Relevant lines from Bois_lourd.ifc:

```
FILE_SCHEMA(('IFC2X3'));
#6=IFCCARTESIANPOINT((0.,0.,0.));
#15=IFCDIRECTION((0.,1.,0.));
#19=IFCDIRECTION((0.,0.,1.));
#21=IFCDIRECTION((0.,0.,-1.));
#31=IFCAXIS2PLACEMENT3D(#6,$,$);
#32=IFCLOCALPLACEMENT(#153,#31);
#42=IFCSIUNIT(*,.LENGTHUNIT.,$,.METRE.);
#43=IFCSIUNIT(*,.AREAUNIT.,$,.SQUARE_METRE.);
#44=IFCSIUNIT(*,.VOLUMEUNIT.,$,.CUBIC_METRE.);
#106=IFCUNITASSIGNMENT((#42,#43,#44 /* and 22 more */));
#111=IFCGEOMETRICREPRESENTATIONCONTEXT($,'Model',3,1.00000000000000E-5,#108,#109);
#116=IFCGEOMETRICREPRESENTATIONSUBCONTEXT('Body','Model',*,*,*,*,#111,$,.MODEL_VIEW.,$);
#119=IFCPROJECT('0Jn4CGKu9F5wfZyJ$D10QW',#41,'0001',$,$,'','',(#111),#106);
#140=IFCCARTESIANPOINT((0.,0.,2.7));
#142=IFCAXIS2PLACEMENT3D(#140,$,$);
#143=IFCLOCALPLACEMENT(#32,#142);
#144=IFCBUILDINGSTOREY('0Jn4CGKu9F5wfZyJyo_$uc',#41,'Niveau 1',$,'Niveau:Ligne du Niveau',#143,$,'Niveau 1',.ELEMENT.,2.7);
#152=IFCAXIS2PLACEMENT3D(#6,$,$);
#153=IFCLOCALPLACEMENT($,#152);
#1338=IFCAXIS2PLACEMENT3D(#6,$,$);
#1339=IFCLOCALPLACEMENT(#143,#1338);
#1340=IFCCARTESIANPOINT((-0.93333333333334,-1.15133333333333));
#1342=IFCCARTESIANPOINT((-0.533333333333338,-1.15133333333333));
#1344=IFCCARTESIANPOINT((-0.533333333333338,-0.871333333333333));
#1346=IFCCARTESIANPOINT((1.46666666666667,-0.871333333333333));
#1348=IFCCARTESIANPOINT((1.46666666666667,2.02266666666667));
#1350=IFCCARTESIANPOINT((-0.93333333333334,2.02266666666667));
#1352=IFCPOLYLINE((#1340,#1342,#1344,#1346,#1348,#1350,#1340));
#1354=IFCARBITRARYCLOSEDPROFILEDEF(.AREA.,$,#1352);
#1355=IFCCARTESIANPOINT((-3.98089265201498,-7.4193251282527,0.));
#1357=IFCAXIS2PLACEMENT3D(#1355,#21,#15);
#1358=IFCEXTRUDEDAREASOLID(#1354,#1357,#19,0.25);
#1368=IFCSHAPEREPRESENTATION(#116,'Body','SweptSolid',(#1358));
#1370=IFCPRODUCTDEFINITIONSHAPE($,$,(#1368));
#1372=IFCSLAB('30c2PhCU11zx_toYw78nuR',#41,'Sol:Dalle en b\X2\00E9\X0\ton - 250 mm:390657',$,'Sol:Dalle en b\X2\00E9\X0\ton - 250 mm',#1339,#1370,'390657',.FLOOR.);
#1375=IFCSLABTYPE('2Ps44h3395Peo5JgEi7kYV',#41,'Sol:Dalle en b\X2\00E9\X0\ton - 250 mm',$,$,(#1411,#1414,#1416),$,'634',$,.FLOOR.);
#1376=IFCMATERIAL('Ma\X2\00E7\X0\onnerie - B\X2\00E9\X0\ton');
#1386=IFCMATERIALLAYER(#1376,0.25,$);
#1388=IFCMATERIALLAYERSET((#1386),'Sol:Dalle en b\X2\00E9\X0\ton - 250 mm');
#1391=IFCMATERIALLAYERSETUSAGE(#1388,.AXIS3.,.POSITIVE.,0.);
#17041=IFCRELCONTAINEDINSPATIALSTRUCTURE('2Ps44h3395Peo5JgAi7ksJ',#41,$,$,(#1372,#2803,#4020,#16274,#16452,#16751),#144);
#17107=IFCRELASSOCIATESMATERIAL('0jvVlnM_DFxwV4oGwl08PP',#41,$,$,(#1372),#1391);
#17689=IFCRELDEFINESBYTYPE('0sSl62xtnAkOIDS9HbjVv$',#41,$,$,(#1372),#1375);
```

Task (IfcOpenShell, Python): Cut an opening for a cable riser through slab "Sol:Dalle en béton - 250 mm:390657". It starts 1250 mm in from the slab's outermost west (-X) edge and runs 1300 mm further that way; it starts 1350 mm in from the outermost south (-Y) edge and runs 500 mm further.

```python
import numpy as np
import ifcopenshell
import ifcopenshell.api.feature
import ifcopenshell.api.geometry
import ifcopenshell.api.root
import ifcopenshell.geom
import ifcopenshell.util.placement
import ifcopenshell.util.representation
import ifcopenshell.util.shape
import ifcopenshell.util.unit

model = ifcopenshell.open("Bois_lourd.ifc")
unit_scale = ifcopenshell.util.unit.calculate_unit_scale(model)
settings = ifcopenshell.geom.settings()


def volume(element):
    """Net volume in cubic metres, openings subtracted."""
    shape = ifcopenshell.geom.create_shape(settings, element)
    return ifcopenshell.util.shape.get_volume(shape.geometry)


slab = model.by_guid("30c2PhCU11zx_toYw78nuR")
before = volume(slab)

# Extent in the slab's own axes, in metres. The edges named are its -X and -Y sides.
slab_shape = ifcopenshell.geom.create_shape(settings, slab)
vertices = ifcopenshell.util.shape.get_vertices(slab_shape.geometry)
x_min, y_min, bottom = vertices.min(axis=0)
top = vertices[:, 2].max()

opening = ifcopenshell.api.root.create_entity(model, ifc_class="IfcOpeningElement", name="Cable riser opening")
context = ifcopenshell.util.representation.get_context(model, "Model", "Body", "MODEL_VIEW")
width, depth = 1.3, 0.5
outline = [(0.0, 0.0), (width, 0.0), (width, depth), (0.0, depth), (0.0, 0.0)]
# Overshoot both faces by 50 mm so the cut is clean.
shape = ifcopenshell.api.geometry.add_slab_representation(
    model, context=context, depth=top - bottom + 0.1, polyline=outline
)
ifcopenshell.api.geometry.assign_representation(model, product=opening, representation=shape)

matrix = ifcopenshell.util.placement.get_local_placement(slab.ObjectPlacement)
matrix[:, 3] = matrix @ np.append(np.array([x_min + 1.25, y_min + 1.35, bottom - 0.05]) / unit_scale, 1.0)
ifcopenshell.api.geometry.edit_object_placement(model, product=opening, matrix=matrix, is_si=False)
ifcopenshell.api.feature.add_feature(model, feature=opening, element=slab)

after = volume(slab)

print(f"slab volume {before:.3f} -> {after:.3f} m3")

model.write("Bois_lourd_edited.ifc")
```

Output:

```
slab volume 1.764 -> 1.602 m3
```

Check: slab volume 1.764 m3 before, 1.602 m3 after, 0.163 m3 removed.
